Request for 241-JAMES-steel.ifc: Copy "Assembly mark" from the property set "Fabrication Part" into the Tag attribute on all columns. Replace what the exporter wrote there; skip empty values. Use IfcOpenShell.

First a look at what the model holds.

```python
import ifcopenshell
import ifcopenshell.util.element

model = ifcopenshell.open("241-JAMES-steel.ifc")
print(model.schema)
columns = model.by_type("IfcColumn")
print(len(columns), "columns")
for e in columns[:8]:
    source = ifcopenshell.util.element.get_pset(e, "Fabrication Part", "Assembly mark")
    target = e.Tag
    print(e.id(), repr(source), repr(target), sep=" | ")
```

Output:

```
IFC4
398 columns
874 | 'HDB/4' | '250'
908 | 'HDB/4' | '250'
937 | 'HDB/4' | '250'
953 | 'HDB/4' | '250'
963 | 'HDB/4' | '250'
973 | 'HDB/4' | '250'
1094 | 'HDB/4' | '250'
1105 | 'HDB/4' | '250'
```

```python
import ifcopenshell
import ifcopenshell.util.element

model = ifcopenshell.open("241-JAMES-steel.ifc")

count = 0
for e in model.by_type("IfcColumn"):
    value = ifcopenshell.util.element.get_pset(e, "Fabrication Part", "Assembly mark")
    current = e.Tag
    if not value or not value.strip() or current == value:
        continue
    e.Tag = value
    count += 1

print(count, "columns updated")

model.write("241-JAMES-steel_updated.ifc")
```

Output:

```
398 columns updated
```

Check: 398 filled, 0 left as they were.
